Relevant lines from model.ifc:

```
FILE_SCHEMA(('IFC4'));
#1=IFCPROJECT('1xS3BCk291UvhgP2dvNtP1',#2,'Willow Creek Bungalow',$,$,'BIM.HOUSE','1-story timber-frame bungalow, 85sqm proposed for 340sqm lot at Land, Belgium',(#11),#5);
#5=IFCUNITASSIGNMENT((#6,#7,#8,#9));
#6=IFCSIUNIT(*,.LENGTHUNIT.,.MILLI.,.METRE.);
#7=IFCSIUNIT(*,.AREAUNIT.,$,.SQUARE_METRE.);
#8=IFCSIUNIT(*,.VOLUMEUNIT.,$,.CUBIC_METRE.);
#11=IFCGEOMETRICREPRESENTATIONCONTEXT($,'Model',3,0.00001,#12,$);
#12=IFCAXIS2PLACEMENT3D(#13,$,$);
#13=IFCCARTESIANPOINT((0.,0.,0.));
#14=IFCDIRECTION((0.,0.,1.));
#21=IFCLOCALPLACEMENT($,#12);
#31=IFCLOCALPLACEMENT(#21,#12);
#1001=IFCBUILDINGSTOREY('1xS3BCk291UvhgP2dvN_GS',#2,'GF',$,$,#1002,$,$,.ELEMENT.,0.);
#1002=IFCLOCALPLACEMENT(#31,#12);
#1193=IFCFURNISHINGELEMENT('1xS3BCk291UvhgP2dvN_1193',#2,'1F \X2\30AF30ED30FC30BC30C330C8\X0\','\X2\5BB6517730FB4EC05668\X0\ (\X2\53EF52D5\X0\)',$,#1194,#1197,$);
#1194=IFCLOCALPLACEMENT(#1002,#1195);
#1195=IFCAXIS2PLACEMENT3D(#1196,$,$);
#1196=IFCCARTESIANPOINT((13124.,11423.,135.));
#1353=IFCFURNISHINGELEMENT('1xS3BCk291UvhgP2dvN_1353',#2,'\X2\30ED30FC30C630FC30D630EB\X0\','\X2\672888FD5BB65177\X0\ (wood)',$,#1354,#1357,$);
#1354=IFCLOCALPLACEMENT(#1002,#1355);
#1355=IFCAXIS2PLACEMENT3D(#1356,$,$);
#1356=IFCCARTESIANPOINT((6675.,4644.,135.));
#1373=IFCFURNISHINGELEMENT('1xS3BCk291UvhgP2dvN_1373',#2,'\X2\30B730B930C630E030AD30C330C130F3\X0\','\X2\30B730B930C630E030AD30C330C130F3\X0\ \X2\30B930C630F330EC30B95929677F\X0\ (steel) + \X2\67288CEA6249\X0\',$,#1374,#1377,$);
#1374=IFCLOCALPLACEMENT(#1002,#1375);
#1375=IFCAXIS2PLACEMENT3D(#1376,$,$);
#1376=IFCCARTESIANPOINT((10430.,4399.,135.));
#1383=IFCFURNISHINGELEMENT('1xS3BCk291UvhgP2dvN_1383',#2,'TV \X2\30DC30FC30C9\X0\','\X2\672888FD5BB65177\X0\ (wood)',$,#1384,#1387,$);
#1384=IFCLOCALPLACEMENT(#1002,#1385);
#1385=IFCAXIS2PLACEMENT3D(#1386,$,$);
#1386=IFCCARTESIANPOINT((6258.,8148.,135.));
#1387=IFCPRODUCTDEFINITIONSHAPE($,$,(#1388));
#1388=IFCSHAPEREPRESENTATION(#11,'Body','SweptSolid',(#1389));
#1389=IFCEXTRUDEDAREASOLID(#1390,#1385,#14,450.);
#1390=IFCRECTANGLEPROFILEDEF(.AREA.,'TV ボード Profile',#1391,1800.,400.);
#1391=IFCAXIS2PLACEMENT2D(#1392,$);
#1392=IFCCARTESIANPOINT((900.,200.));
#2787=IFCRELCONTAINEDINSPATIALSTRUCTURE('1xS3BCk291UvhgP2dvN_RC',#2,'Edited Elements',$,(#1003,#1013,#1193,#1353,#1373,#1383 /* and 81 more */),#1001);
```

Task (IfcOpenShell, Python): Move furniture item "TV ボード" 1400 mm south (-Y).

```python
import ifcopenshell
import ifcopenshell.api.geometry
import ifcopenshell.util.placement

model = ifcopenshell.open("model.ifc")

item = model.by_guid("1xS3BCk291UvhgP2dvN_1383")
matrix = ifcopenshell.util.placement.get_local_placement(item.ObjectPlacement)
matrix[1, 3] -= 1400.0
ifcopenshell.api.geometry.edit_object_placement(model, product=item, matrix=matrix, is_si=False)

print(ifcopenshell.util.placement.get_local_placement(item.ObjectPlacement).round(3) + 0.0)

model.write("model_updated.ifc")
```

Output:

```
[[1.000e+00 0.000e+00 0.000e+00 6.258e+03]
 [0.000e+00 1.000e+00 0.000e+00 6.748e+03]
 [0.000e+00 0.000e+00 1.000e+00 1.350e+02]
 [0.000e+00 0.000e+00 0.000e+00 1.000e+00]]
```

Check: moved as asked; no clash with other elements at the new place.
